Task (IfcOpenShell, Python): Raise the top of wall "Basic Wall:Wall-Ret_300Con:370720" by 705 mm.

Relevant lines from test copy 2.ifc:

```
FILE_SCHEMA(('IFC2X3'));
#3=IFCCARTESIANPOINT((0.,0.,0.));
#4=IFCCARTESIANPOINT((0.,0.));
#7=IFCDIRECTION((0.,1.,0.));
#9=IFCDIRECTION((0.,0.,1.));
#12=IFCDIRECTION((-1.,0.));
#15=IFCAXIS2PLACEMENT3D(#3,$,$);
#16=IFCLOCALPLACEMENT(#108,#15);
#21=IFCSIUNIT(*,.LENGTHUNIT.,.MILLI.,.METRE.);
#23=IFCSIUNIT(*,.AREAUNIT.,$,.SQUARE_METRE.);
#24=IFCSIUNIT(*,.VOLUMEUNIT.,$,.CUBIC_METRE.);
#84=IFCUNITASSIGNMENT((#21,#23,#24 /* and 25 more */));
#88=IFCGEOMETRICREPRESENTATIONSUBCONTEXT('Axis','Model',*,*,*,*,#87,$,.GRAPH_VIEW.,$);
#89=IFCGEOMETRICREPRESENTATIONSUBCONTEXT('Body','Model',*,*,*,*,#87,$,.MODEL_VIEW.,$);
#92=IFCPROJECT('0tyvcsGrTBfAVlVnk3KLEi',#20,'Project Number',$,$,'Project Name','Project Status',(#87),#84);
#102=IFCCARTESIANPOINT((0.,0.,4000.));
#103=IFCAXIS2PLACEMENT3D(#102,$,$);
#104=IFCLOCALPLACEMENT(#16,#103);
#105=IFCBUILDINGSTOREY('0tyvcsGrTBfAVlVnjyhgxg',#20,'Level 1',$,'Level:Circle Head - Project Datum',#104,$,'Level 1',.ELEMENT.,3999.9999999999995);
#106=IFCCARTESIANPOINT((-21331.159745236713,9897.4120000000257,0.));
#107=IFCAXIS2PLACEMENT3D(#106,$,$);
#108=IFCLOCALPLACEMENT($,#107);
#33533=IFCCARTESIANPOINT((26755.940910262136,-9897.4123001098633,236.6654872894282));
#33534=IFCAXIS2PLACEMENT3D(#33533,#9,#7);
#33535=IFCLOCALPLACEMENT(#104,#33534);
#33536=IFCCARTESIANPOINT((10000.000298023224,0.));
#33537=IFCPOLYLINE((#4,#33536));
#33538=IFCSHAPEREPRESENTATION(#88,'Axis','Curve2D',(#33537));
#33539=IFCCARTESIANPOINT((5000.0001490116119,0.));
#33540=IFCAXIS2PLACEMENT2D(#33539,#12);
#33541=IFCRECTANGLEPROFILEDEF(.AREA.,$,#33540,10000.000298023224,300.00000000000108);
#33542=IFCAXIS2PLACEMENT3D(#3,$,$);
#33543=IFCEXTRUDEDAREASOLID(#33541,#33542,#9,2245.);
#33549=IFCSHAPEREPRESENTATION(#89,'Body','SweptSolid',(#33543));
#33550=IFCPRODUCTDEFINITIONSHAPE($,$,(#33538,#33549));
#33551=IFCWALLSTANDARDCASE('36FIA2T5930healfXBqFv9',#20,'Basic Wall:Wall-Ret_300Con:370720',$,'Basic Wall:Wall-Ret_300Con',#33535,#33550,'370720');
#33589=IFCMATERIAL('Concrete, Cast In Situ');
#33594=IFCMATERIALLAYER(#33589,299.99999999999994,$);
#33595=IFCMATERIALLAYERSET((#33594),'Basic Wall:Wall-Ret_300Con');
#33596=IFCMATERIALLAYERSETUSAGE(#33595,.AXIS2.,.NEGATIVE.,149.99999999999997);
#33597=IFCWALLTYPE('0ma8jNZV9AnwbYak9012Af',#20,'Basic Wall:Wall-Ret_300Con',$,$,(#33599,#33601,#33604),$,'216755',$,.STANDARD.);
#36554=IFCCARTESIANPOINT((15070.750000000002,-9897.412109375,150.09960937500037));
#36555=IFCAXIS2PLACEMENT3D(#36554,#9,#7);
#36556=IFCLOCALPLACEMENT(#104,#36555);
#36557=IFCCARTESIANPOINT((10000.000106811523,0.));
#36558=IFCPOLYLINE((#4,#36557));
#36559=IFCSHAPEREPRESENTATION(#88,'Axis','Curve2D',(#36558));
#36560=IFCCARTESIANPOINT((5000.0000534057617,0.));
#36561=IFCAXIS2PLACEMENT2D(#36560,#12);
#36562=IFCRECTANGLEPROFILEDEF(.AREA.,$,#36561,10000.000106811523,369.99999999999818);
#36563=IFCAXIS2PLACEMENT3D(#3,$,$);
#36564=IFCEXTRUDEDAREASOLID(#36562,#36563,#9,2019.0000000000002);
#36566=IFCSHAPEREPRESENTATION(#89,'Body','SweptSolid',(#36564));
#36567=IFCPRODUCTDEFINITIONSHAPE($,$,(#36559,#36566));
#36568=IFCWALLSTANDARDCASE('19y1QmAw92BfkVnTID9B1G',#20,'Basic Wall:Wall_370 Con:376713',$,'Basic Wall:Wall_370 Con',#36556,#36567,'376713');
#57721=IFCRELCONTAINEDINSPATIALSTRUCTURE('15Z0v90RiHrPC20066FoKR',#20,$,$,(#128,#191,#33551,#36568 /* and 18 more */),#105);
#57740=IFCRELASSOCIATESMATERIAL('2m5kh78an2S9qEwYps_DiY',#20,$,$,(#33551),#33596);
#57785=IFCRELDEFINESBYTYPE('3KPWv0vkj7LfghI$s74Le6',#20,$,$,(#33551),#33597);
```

```python
import ifcopenshell
import ifcopenshell.geom
import ifcopenshell.util.representation
import ifcopenshell.util.shape
import ifcopenshell.util.unit

model = ifcopenshell.open("test copy 2.ifc")
unit_scale = ifcopenshell.util.unit.calculate_unit_scale(model)
settings = ifcopenshell.geom.settings()


def volume(element):
    """Net volume in cubic metres, openings subtracted."""
    shape = ifcopenshell.geom.create_shape(settings, element)
    return ifcopenshell.util.shape.get_volume(shape.geometry)


wall = model.by_guid("36FIA2T5930healfXBqFv9")
before = volume(wall)

body = ifcopenshell.util.representation.get_representation(wall, "Model", "Body")
solid = body.Items[0]
old_height = solid.Depth
solid.Depth += 0.705 / unit_scale
after = volume(wall)

print(f"height {old_height:g} -> {solid.Depth:g}, volume {before:.3f} -> {after:.3f} m3")

model.write("test copy 2-out.ifc")
```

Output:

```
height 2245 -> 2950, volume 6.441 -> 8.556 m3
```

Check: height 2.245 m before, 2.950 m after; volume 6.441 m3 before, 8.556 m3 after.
